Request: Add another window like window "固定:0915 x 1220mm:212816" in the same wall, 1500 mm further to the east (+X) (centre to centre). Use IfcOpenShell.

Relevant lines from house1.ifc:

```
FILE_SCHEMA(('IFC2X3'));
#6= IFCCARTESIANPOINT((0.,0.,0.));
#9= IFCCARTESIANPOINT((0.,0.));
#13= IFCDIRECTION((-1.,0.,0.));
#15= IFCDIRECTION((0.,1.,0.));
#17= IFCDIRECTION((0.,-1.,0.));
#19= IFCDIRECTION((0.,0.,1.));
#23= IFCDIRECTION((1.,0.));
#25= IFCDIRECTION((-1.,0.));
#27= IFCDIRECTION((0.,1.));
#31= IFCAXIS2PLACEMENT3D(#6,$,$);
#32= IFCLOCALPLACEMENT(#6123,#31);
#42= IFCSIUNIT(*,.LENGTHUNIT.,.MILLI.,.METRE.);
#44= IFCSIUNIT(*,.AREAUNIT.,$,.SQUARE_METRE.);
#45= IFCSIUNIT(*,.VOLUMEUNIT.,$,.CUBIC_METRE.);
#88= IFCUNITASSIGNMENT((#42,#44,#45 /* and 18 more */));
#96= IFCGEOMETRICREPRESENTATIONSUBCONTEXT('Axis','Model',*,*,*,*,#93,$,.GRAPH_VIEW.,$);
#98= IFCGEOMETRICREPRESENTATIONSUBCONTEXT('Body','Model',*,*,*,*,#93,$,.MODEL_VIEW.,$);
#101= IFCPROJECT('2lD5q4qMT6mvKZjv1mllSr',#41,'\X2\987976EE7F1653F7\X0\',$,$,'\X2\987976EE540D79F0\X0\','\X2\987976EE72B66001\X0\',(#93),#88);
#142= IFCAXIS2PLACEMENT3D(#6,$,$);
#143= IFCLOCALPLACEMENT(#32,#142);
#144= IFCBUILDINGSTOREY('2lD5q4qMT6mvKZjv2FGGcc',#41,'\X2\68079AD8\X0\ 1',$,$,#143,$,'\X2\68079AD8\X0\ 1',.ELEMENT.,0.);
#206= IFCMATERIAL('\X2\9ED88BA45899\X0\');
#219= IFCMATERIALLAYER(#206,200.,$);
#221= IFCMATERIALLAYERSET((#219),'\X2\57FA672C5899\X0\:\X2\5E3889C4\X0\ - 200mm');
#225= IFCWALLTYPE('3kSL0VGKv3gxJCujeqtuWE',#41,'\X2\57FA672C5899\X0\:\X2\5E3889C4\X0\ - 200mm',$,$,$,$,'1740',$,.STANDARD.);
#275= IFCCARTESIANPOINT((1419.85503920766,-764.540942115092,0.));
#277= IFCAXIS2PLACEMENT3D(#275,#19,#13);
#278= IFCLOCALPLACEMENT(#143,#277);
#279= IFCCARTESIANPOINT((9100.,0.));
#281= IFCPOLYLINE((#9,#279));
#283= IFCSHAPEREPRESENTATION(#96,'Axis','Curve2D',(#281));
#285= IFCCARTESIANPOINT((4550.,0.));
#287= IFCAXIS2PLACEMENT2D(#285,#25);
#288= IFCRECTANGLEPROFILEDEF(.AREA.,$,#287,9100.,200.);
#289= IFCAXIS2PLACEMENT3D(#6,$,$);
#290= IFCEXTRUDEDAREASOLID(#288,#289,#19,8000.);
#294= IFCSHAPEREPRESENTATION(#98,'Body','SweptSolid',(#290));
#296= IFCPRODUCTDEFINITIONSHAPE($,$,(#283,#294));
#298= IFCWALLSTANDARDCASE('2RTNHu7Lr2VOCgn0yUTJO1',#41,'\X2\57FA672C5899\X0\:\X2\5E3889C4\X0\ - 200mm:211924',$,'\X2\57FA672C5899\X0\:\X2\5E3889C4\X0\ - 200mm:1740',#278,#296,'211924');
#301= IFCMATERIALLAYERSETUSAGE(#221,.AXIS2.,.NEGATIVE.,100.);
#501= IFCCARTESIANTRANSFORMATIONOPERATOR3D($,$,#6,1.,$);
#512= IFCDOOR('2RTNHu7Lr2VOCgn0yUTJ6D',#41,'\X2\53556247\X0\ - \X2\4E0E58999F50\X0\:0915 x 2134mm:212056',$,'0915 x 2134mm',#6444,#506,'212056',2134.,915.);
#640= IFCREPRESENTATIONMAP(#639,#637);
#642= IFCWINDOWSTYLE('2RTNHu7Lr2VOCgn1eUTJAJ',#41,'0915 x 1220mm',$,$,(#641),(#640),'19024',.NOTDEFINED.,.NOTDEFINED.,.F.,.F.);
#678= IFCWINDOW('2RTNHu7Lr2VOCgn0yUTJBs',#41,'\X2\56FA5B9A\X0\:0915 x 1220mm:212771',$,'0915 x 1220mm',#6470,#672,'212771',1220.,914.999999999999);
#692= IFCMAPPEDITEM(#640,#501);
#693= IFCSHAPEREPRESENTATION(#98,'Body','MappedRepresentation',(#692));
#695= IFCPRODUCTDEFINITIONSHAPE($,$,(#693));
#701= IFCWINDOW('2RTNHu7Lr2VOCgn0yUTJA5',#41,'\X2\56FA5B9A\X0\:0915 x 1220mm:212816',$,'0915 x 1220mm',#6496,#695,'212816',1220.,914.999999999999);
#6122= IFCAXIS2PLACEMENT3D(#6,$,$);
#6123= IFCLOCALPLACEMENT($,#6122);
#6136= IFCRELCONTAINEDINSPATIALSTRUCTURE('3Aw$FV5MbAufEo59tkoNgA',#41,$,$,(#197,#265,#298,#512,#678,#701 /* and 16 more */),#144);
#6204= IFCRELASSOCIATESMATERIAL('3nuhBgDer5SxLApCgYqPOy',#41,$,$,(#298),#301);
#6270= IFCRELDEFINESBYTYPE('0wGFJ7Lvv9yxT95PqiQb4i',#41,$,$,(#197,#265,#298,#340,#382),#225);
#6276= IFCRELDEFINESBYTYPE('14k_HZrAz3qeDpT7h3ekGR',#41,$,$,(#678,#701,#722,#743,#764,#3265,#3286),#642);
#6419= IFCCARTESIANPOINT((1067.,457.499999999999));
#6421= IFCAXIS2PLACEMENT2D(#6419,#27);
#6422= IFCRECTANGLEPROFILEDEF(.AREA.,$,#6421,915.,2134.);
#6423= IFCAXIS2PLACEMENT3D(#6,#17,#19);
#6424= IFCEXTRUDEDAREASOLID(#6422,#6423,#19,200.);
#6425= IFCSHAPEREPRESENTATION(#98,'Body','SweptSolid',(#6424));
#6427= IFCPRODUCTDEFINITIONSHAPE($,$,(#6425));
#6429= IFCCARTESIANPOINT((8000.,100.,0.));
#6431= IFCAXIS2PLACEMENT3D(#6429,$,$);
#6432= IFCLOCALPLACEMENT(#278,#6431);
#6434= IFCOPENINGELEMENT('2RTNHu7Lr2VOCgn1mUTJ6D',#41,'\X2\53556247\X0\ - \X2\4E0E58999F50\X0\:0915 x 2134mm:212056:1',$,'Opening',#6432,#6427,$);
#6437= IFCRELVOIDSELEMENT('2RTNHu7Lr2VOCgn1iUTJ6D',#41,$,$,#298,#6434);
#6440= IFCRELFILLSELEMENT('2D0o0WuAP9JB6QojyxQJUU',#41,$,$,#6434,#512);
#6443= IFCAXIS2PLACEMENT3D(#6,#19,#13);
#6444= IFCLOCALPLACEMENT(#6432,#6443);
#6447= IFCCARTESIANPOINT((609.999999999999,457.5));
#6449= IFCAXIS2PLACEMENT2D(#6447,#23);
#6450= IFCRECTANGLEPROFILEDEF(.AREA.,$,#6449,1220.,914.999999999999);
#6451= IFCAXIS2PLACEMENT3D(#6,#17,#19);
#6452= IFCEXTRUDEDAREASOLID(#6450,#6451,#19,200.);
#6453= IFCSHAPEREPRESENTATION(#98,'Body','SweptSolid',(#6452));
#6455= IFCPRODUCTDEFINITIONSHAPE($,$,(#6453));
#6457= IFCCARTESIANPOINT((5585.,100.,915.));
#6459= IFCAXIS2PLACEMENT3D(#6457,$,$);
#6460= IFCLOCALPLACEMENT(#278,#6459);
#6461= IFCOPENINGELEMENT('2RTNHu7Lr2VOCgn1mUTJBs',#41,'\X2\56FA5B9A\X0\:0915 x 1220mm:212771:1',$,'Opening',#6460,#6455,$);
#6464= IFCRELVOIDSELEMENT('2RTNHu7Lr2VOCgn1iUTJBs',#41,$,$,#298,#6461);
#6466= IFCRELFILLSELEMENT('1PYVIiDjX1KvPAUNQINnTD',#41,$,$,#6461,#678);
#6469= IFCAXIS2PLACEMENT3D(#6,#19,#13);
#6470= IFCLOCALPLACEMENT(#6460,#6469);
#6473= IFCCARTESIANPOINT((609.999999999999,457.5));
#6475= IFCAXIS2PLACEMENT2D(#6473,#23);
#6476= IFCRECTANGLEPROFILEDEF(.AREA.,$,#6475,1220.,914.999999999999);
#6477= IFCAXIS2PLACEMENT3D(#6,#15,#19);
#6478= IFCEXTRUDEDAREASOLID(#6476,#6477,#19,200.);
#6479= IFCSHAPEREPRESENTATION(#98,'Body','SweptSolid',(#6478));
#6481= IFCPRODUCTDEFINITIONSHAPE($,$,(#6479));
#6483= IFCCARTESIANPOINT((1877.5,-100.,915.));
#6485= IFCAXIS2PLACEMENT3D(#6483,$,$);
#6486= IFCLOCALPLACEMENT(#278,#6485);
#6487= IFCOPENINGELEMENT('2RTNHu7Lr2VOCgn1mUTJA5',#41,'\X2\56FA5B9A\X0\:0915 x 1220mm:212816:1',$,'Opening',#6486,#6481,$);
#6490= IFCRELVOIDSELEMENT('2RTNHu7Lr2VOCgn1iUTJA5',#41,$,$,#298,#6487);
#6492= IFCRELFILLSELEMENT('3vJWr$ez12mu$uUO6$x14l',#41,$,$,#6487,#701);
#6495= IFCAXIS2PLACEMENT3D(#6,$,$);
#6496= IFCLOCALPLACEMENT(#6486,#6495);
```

```python
import ifcopenshell
import ifcopenshell.api.feature
import ifcopenshell.api.geometry
import ifcopenshell.api.root
import ifcopenshell.geom
import ifcopenshell.util.element
import ifcopenshell.util.placement
import ifcopenshell.util.shape
import ifcopenshell.util.unit

model = ifcopenshell.open("house1.ifc")
unit_scale = ifcopenshell.util.unit.calculate_unit_scale(model)
settings = ifcopenshell.geom.settings()


def volume(element):
    """Net volume in cubic metres, openings subtracted."""
    shape = ifcopenshell.geom.create_shape(settings, element)
    return ifcopenshell.util.shape.get_volume(shape.geometry)


def reuse_history(source, copy):
    """copy_class also copies each property set's owner history, people and application; keep the originals."""
    for rel in copy.IsDefinedBy:
        if rel.is_a("IfcRelDefinesByProperties") and (history := rel.RelatingPropertyDefinition.OwnerHistory):
            rel.RelatingPropertyDefinition.OwnerHistory = source.OwnerHistory
            ifcopenshell.util.element.remove_deep2(model, history)


window = model.by_guid("2RTNHu7Lr2VOCgn0yUTJA5")
opening = window.FillsVoids[0].RelatingOpeningElement
wall = opening.VoidsElements[0].RelatingBuildingElement
before = volume(wall)
shift = ifcopenshell.util.placement.get_local_placement(wall.ObjectPlacement)[:3, 0] * -1.5 / unit_scale

# copy_class copies the void relationship, type, container and properties, but no geometry.
new_opening = ifcopenshell.api.root.copy_class(model, product=opening)
new_opening.Representation = ifcopenshell.util.element.copy_deep(
    model, opening.Representation, exclude=["IfcGeometricRepresentationContext", "IfcRepresentationMap"]
)
new_opening.Name = "固定:0915 x 1220mm"
new_window = ifcopenshell.api.root.copy_class(model, product=window)
new_window.Representation = ifcopenshell.util.element.copy_deep(
    model, window.Representation, exclude=["IfcGeometricRepresentationContext", "IfcRepresentationMap"]
)
new_window.Name = "固定:0915 x 1220mm"
new_window.Tag = None
reuse_history(window, new_window)
fills = ifcopenshell.api.feature.add_filling(model, opening=new_opening, element=new_window)
fills.OwnerHistory = new_window.OwnerHistory  # required in IFC2X3

for old, new in ((opening, new_opening), (window, new_window)):
    matrix = ifcopenshell.util.placement.get_local_placement(old.ObjectPlacement)
    matrix[:3, 3] += shift
    ifcopenshell.api.geometry.edit_object_placement(model, product=new, matrix=matrix, is_si=False)

after = volume(wall)

print(f"wall volume {before:.3f} -> {after:.3f} m3")

model.write("house1_v2.ifc")
```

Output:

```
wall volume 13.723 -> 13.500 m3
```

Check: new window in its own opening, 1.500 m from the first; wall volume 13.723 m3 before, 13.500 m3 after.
